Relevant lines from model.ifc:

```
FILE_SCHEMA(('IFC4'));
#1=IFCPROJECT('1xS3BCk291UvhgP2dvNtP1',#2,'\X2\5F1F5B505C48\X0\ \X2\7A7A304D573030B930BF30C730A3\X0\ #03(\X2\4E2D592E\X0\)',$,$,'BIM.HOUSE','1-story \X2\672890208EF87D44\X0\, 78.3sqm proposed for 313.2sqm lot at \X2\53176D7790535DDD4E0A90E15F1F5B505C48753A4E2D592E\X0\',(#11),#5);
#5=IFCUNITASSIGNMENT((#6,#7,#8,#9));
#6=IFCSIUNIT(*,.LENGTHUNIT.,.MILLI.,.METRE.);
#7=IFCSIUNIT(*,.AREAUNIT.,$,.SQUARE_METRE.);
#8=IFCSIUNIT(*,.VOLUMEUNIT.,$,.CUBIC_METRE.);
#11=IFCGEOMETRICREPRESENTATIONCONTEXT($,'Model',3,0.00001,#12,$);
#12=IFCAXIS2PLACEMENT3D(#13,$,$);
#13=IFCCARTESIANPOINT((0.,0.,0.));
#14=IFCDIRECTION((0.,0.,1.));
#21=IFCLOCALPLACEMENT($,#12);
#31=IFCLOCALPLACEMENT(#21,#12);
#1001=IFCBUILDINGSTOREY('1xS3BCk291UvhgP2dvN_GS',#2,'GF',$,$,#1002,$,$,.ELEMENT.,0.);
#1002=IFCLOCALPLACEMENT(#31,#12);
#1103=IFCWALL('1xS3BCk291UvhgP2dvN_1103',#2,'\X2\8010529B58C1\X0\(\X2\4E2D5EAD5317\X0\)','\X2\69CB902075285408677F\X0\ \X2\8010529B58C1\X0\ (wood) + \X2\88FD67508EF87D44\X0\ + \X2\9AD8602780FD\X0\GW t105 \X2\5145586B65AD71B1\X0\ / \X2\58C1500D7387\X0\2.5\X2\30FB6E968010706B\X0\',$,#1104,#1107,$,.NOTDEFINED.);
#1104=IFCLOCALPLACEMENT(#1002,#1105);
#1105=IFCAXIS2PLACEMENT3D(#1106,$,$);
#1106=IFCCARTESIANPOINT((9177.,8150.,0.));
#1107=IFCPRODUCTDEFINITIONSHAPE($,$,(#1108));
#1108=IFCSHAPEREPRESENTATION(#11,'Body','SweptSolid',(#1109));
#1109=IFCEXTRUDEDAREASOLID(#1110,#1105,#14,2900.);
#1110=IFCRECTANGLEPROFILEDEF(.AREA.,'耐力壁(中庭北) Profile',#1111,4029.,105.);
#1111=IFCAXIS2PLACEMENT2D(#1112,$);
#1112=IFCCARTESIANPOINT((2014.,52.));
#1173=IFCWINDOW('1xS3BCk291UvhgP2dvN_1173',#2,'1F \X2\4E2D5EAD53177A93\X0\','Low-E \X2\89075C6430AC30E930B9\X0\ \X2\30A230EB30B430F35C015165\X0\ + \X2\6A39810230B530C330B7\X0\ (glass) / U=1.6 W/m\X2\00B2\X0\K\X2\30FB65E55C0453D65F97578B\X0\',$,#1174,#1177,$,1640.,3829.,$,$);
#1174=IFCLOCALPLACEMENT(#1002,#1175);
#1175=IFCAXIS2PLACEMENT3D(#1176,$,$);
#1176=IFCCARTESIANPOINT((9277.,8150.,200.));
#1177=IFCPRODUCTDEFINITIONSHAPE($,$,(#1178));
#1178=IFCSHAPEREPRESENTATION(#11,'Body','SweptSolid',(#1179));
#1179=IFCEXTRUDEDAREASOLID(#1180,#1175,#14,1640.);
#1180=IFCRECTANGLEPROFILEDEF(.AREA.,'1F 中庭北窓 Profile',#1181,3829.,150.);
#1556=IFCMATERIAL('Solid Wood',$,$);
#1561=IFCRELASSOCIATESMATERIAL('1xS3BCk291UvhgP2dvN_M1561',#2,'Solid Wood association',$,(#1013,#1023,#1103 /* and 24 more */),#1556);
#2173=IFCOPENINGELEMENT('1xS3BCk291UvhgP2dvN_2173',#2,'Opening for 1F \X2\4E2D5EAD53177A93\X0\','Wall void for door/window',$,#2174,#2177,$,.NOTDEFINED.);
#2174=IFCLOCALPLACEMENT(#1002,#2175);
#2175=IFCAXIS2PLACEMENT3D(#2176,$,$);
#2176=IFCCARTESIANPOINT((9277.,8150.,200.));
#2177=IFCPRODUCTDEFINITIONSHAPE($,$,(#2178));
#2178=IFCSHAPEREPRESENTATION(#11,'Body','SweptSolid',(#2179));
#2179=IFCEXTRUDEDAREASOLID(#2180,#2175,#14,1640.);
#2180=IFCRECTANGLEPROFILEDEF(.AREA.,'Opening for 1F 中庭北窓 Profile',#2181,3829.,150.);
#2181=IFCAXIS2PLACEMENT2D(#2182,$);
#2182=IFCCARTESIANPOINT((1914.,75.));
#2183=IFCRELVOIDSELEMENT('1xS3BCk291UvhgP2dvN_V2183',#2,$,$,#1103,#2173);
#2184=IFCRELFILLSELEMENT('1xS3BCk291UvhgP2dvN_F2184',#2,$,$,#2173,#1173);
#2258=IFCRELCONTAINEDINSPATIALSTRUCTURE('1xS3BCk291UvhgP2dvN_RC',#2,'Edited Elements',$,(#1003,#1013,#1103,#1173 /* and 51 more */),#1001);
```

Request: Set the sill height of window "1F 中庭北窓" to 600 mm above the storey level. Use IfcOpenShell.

```python
import numpy as np
import ifcopenshell
import ifcopenshell.api.geometry
import ifcopenshell.geom
import ifcopenshell.util.element
import ifcopenshell.util.placement
import ifcopenshell.util.shape
import ifcopenshell.util.unit

model = ifcopenshell.open("model.ifc")
unit_scale = ifcopenshell.util.unit.calculate_unit_scale(model)

window = model.by_guid("1xS3BCk291UvhgP2dvN_1173")
opening = window.FillsVoids[0].RelatingOpeningElement
storey = ifcopenshell.util.element.get_container(window, ifc_class="IfcBuildingStorey")
level = ifcopenshell.util.placement.get_local_placement(storey.ObjectPlacement)[2, 3]

# The opening's origin need not be at the sill, so measure its lowest point.
shape = ifcopenshell.geom.create_shape(ifcopenshell.geom.settings(), opening)
bottom = ifcopenshell.util.shape.get_shape_bottom_elevation(shape, shape.geometry) / unit_scale
dz = level + 600.0 - bottom

shift = np.array([0.0, 0.0, dz])
# The window is not placed relative to its opening, so move both.
for product in (opening, window):
    matrix = ifcopenshell.util.placement.get_local_placement(product.ObjectPlacement)
    matrix[:3, 3] += shift
    ifcopenshell.api.geometry.edit_object_placement(model, product=product, matrix=matrix, is_si=False)

print(f"moved by {dz * unit_scale:+.3f} m")

model.write("model_v2.ifc")
```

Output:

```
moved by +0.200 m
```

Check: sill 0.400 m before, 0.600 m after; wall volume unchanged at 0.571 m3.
